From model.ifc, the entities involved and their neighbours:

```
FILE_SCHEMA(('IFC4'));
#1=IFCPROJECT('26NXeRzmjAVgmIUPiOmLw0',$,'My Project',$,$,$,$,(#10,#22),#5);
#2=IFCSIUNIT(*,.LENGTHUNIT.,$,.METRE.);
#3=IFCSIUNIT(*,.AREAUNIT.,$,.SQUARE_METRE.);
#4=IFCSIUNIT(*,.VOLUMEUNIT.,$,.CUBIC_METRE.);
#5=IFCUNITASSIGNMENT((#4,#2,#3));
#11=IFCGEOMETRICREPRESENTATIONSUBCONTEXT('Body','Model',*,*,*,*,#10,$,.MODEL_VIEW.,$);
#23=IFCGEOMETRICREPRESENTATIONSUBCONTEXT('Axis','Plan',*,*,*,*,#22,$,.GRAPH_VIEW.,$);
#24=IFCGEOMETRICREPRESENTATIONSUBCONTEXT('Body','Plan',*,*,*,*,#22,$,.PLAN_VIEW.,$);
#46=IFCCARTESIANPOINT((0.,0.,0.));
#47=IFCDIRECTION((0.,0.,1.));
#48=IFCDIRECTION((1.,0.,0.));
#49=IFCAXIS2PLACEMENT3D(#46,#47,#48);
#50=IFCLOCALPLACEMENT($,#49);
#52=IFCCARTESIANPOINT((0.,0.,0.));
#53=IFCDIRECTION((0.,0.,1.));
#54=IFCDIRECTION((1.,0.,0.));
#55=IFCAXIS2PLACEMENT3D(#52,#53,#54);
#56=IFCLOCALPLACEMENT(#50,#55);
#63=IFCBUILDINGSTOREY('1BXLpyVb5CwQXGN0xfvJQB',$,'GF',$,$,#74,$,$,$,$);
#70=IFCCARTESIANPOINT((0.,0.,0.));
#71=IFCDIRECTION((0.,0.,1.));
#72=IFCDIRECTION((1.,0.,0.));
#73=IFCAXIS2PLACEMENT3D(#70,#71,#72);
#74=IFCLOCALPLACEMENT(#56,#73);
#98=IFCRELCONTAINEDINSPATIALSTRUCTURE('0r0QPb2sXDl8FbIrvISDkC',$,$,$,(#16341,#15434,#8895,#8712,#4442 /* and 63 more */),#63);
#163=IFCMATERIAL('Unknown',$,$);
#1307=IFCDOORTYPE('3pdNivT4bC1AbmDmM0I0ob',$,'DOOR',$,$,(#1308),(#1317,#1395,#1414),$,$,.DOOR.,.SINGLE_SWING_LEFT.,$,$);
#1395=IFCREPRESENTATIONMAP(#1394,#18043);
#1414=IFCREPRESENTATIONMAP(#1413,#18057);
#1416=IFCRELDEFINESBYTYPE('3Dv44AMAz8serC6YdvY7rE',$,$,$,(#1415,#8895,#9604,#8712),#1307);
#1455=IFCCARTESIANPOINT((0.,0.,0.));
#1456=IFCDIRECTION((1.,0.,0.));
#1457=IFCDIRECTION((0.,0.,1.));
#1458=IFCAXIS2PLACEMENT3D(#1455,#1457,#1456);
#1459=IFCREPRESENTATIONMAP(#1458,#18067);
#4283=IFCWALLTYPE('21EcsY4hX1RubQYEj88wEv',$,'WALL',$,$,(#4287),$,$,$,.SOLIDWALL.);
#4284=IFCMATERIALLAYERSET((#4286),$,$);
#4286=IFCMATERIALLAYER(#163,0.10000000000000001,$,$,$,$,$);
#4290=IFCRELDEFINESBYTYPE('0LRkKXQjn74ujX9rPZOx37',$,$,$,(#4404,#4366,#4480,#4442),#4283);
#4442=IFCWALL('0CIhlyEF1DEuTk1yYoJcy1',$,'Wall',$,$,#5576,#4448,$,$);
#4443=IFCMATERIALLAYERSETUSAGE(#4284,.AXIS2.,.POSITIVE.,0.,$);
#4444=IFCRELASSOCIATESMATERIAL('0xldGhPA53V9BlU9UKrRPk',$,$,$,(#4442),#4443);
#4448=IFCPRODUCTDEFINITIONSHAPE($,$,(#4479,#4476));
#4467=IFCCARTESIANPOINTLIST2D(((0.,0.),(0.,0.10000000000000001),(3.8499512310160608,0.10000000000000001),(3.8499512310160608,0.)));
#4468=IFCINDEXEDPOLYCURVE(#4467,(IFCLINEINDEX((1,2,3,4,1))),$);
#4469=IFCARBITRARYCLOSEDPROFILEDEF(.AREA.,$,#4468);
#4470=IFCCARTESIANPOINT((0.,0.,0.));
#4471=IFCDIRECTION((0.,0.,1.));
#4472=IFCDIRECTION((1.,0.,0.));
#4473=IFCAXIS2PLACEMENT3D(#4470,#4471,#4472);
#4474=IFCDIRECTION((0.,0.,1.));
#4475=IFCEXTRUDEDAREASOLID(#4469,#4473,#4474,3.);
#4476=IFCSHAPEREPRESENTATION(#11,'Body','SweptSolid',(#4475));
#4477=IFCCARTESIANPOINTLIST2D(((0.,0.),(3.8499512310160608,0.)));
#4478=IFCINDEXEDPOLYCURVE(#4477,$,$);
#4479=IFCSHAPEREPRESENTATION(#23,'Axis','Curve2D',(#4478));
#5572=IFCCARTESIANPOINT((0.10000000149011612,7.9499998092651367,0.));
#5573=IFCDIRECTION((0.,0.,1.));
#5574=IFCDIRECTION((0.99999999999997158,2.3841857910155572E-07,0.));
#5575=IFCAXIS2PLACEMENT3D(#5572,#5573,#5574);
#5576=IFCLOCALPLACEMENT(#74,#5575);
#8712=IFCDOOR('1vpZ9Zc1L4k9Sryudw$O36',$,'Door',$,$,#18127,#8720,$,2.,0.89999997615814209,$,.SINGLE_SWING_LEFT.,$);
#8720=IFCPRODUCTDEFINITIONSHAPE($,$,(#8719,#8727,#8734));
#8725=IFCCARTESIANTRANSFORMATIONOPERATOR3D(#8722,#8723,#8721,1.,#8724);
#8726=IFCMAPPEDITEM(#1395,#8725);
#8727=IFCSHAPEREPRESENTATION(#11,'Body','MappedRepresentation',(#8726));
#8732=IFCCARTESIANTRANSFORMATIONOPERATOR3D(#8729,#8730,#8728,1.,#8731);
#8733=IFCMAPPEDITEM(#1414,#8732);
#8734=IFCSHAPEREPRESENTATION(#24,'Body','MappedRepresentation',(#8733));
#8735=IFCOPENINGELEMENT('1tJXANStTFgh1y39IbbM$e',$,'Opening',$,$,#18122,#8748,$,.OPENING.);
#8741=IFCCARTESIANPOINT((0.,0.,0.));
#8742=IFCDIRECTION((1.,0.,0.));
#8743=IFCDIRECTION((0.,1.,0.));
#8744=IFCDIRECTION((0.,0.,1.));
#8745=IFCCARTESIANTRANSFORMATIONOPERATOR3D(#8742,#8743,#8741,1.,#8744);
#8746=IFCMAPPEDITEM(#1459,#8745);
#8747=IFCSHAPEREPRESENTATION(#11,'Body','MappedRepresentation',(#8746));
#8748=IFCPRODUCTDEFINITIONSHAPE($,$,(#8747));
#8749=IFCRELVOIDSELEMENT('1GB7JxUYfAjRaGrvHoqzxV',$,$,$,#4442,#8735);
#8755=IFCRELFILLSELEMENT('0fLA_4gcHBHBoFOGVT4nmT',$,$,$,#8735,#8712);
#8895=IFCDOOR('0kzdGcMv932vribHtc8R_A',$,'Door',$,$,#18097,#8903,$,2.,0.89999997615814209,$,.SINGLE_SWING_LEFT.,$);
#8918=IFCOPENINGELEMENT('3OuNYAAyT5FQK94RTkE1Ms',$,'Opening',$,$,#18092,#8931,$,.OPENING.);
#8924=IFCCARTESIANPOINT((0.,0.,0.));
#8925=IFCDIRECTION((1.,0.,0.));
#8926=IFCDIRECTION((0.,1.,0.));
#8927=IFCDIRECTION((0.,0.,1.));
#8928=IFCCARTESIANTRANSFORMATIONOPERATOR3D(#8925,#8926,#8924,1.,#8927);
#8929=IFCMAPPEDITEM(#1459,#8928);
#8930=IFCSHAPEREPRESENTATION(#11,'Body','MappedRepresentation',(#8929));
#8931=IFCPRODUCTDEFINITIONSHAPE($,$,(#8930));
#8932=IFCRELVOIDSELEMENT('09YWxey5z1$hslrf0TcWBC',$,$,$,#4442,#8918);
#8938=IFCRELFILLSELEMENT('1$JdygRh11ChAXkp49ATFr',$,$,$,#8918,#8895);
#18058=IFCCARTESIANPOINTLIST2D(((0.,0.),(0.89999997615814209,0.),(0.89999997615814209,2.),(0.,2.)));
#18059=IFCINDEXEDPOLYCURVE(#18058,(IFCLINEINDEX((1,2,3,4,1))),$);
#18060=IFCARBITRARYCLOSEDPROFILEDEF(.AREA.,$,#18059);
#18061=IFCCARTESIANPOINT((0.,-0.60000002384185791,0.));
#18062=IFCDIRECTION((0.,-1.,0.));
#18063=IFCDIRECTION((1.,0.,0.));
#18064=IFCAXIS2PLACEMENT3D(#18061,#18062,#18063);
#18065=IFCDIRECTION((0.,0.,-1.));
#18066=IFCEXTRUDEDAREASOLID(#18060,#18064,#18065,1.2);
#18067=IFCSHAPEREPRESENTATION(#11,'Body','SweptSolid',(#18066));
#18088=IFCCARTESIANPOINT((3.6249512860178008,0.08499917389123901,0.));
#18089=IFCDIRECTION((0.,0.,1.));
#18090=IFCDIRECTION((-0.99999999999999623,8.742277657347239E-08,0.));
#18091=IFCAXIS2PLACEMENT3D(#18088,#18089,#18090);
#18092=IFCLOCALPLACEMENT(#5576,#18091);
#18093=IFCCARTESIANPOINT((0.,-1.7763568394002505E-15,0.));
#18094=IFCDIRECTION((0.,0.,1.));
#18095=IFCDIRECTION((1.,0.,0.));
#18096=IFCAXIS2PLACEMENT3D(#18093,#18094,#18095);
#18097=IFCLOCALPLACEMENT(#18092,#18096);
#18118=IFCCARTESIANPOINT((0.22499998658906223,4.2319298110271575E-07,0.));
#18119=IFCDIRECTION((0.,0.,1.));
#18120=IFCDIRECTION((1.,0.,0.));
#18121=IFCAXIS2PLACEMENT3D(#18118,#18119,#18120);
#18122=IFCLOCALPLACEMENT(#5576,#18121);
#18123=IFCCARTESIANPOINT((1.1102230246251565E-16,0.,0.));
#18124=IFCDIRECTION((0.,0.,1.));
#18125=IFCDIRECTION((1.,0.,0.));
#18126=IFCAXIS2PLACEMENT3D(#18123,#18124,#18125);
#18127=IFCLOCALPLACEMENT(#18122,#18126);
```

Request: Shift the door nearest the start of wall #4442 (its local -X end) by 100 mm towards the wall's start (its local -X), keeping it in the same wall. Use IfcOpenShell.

```python
import ifcopenshell
import ifcopenshell.api.geometry
import ifcopenshell.util.placement

model = ifcopenshell.open("model.ifc")

door = model.by_guid("1vpZ9Zc1L4k9Sryudw$O36")
opening = door.FillsVoids[0].RelatingOpeningElement
wall = opening.VoidsElements[0].RelatingBuildingElement

wall_matrix = ifcopenshell.util.placement.get_local_placement(wall.ObjectPlacement)
shift = wall_matrix[:3, 0] * -0.1
before = ifcopenshell.util.placement.get_local_placement(door.ObjectPlacement)[:3, 3].copy()

# The door is placed relative to its opening, so it follows when the opening moves.
matrix = ifcopenshell.util.placement.get_local_placement(opening.ObjectPlacement)
matrix[:3, 3] += shift
ifcopenshell.api.geometry.edit_object_placement(
    model, product=opening, matrix=matrix, is_si=False, should_transform_children=True
)

after = ifcopenshell.util.placement.get_local_placement(door.ObjectPlacement)[:3, 3]
print("door moved by", (after - before).round(3) + 0.0)

model.write("model_updated.ifc")
```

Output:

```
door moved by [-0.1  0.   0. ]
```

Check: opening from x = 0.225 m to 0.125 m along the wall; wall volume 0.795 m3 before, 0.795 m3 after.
